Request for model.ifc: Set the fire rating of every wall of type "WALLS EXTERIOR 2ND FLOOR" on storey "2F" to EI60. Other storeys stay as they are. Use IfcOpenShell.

First a look at what the model holds.

```python
import ifcopenshell
import ifcopenshell.util.element

model = ifcopenshell.open("model.ifc")
print(model.schema)
storey = next(s for s in model.by_type("IfcBuildingStorey") if s.Name == "2F")
walls = [e for e in ifcopenshell.util.element.get_decomposition(storey) if e.is_a("IfcWall")]
seen = {}
for e in walls:
    element_type = ifcopenshell.util.element.get_type(e)
    key = (element_type.Name if element_type != e and element_type else None, ifcopenshell.util.element.get_pset(e, "Pset_WallCommon", "FireRating"))
    seen[key] = seen.get(key, 0) + 1
for (name, value), count in sorted(seen.items(), key=str):
    print(count, "x", name, "|", value)
```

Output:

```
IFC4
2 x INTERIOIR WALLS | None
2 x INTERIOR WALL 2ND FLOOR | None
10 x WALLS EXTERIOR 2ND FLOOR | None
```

```python
import ifcopenshell
import ifcopenshell.api.pset
import ifcopenshell.util.element

model = ifcopenshell.open("model.ifc")

storey = next(s for s in model.by_type("IfcBuildingStorey") if s.Name == "2F")
walls = [e for e in ifcopenshell.util.element.get_decomposition(storey) if e.is_a("IfcWall")]

count = 0
for e in walls:
    element_type = ifcopenshell.util.element.get_type(e)
    if element_type in (None, e) or element_type.Name != "WALLS EXTERIOR 2ND FLOOR":
        continue
    # add_pset returns the element's existing set when there is one.
    pset = ifcopenshell.api.pset.add_pset(model, product=e, name="Pset_WallCommon")
    ifcopenshell.api.pset.edit_pset(model, pset=pset, properties={"FireRating": "EI60"})
    count += 1

print(count, "walls updated")

model.write("model_updated.ifc")
```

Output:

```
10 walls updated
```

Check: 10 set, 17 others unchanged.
